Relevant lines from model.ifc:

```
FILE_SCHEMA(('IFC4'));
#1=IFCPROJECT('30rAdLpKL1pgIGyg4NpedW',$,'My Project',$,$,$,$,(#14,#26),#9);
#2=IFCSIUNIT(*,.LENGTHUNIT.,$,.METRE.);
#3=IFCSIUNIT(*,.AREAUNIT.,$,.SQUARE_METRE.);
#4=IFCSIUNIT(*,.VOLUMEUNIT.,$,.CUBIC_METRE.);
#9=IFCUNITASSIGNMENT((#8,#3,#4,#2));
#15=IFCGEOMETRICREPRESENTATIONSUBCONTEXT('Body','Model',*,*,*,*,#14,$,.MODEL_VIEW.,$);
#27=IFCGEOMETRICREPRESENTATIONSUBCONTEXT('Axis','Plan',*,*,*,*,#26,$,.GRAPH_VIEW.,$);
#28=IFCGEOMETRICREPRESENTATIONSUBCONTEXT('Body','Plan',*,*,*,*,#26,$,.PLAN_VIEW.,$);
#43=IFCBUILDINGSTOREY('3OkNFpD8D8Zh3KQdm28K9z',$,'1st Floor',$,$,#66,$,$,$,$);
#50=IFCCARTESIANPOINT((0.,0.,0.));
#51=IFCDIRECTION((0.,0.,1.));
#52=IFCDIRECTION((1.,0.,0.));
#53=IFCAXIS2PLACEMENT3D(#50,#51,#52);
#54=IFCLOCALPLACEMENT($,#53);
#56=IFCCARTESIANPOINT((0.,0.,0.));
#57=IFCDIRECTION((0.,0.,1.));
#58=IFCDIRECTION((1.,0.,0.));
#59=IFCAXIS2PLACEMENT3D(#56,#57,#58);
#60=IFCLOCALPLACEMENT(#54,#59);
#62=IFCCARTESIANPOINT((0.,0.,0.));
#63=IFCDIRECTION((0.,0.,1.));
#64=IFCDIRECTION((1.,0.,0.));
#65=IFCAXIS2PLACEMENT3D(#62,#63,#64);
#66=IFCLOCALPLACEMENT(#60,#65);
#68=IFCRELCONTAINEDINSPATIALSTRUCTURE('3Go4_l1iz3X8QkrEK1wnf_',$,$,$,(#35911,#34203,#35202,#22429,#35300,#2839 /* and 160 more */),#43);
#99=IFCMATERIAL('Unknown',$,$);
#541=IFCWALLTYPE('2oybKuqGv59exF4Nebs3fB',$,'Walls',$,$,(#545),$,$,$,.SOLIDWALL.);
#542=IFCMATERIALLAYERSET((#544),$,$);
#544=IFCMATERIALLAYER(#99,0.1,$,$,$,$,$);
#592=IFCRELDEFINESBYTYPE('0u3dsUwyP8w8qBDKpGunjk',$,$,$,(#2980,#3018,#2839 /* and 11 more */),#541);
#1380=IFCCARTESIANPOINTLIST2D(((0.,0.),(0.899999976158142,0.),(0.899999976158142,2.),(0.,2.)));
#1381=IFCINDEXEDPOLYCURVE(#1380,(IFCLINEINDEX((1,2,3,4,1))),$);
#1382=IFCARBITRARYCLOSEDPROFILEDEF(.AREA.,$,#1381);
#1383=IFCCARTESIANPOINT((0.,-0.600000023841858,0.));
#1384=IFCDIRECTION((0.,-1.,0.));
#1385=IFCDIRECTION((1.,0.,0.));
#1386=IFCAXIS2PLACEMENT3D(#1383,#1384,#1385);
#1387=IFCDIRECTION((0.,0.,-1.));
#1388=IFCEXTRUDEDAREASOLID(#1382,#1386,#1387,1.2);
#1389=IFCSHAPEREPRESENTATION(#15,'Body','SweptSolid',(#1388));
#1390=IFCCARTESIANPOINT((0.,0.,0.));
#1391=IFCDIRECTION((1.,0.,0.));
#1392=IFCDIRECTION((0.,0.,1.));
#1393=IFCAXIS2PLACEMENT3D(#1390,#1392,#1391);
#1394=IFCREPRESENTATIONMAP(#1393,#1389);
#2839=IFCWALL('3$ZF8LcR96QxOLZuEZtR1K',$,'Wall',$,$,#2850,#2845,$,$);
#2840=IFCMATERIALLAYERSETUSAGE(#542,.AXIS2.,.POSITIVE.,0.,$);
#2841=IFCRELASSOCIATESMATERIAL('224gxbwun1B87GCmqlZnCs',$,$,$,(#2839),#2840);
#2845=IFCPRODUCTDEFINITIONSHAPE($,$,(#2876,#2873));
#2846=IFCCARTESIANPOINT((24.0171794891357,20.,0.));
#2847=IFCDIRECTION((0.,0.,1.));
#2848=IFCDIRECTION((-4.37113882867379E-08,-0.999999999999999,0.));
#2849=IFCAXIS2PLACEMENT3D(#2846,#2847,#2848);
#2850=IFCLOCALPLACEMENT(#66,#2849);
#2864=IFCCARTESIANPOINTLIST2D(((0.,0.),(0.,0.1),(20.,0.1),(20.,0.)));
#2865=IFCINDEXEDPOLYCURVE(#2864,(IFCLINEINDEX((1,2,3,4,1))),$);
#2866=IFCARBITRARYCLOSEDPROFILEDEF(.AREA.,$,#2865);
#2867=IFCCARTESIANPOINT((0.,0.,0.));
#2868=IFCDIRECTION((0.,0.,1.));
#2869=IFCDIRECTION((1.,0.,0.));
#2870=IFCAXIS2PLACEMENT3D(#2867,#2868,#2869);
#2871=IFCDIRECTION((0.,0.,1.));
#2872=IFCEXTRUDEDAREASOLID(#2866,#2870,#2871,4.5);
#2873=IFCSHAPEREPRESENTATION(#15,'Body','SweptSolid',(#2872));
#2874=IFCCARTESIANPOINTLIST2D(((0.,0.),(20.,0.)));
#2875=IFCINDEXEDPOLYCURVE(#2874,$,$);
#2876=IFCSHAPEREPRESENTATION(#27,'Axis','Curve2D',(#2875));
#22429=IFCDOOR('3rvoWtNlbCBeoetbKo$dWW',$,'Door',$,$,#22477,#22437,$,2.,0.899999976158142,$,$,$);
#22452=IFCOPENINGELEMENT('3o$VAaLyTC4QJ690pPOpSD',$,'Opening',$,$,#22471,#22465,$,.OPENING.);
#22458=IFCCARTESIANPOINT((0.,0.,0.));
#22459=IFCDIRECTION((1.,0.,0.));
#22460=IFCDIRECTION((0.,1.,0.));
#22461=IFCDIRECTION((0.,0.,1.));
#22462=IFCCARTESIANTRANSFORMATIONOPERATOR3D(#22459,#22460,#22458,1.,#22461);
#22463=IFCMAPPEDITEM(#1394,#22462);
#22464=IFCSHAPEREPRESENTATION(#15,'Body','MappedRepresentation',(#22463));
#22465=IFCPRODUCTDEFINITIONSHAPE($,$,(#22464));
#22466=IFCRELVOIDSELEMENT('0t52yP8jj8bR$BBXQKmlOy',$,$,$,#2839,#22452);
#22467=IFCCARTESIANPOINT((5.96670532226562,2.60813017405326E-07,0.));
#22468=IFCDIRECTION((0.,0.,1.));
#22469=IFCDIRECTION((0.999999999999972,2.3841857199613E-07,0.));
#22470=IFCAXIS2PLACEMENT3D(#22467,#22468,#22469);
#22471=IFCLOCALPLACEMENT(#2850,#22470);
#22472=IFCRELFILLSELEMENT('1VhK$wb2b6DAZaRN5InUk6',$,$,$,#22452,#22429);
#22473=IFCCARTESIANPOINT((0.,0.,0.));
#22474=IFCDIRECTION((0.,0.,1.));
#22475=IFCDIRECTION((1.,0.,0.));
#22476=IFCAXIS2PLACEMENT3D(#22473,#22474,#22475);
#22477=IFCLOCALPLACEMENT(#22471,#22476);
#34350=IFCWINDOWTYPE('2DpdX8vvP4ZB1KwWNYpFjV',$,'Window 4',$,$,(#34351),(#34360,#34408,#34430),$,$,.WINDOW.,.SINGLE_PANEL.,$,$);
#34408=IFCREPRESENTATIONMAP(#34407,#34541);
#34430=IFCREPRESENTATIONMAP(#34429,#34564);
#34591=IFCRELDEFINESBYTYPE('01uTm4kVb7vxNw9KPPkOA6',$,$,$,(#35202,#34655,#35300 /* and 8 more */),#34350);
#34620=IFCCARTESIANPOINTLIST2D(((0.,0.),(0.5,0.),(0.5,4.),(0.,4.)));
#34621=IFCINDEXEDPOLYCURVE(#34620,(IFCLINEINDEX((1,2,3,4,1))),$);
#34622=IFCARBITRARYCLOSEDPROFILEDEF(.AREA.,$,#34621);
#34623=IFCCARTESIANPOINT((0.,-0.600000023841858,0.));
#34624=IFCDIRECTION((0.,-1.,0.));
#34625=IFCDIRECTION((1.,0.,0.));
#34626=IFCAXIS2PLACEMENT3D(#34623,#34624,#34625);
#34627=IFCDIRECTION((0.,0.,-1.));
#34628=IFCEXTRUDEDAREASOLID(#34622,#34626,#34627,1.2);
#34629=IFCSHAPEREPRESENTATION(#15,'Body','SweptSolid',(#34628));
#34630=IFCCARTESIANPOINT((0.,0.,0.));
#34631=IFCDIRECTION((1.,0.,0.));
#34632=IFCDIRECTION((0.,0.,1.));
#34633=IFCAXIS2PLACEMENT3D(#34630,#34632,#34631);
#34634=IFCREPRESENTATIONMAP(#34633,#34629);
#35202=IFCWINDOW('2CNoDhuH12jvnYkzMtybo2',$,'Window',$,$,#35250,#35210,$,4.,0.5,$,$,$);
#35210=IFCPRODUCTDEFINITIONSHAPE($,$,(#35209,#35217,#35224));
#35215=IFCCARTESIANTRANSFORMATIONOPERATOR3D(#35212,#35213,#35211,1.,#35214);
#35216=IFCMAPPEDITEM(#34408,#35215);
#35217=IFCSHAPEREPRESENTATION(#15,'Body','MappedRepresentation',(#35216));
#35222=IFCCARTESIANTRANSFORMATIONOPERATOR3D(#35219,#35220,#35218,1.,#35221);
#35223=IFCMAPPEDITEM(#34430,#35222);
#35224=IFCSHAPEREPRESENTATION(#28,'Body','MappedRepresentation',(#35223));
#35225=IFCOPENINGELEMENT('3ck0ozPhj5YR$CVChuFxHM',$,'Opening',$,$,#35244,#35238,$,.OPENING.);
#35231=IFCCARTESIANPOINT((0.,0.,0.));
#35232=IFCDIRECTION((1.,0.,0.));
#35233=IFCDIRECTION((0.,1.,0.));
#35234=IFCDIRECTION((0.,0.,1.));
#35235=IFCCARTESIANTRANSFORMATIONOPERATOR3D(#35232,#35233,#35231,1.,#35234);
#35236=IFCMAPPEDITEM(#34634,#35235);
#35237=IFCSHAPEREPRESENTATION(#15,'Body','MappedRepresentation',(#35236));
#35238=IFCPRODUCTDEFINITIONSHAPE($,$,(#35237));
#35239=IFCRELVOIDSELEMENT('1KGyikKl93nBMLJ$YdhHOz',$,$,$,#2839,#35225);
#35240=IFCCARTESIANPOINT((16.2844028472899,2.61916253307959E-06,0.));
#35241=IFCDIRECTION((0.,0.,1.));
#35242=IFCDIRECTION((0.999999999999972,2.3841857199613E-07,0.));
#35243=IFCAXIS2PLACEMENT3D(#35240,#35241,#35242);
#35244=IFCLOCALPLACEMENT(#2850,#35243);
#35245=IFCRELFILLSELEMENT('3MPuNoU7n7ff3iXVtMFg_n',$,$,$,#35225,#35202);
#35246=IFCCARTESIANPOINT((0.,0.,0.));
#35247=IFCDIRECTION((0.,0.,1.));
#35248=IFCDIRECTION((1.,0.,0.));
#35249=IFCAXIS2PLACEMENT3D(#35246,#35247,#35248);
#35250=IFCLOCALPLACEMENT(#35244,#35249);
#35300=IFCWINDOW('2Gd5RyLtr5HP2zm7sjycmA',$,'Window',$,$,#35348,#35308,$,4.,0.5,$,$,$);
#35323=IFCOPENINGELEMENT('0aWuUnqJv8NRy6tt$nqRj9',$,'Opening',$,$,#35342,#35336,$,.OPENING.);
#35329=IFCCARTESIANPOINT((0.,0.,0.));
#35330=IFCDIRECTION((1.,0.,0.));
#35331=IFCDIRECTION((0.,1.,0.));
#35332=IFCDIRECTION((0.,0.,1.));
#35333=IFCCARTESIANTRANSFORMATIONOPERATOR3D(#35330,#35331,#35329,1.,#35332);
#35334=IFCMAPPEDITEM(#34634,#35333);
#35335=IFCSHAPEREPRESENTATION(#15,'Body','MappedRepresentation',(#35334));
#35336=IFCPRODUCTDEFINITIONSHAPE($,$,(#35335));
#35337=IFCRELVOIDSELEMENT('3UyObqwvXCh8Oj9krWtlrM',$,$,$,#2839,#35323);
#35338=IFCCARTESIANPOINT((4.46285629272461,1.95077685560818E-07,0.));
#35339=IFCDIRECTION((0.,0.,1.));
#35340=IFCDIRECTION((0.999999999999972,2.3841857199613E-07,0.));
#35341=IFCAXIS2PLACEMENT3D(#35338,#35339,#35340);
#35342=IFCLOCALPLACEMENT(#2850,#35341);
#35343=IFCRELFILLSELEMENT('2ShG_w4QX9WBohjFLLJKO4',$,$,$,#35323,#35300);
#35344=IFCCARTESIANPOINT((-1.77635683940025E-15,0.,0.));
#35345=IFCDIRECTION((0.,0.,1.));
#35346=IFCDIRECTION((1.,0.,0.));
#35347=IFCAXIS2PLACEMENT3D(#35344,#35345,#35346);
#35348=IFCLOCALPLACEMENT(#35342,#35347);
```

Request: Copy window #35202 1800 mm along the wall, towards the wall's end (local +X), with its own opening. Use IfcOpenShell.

```python
import ifcopenshell
import ifcopenshell.api.feature
import ifcopenshell.api.geometry
import ifcopenshell.api.root
import ifcopenshell.geom
import ifcopenshell.util.element
import ifcopenshell.util.placement
import ifcopenshell.util.shape

model = ifcopenshell.open("model.ifc")
settings = ifcopenshell.geom.settings()


def volume(element):
    """Net volume in cubic metres, openings subtracted."""
    shape = ifcopenshell.geom.create_shape(settings, element)
    return ifcopenshell.util.shape.get_volume(shape.geometry)


window = model.by_guid("2CNoDhuH12jvnYkzMtybo2")
opening = window.FillsVoids[0].RelatingOpeningElement
wall = opening.VoidsElements[0].RelatingBuildingElement
before = volume(wall)
shift = ifcopenshell.util.placement.get_local_placement(wall.ObjectPlacement)[:3, 0] * 1.8

# copy_class copies the void relationship, type, container and properties, but no geometry.
new_opening = ifcopenshell.api.root.copy_class(model, product=opening)
new_opening.Representation = ifcopenshell.util.element.copy_deep(
    model, opening.Representation, exclude=["IfcGeometricRepresentationContext", "IfcRepresentationMap"]
)
new_window = ifcopenshell.api.root.copy_class(model, product=window)
new_window.Representation = ifcopenshell.util.element.copy_deep(
    model, window.Representation, exclude=["IfcGeometricRepresentationContext", "IfcRepresentationMap"]
)
ifcopenshell.api.feature.add_filling(model, opening=new_opening, element=new_window)

for old, new in ((opening, new_opening), (window, new_window)):
    matrix = ifcopenshell.util.placement.get_local_placement(old.ObjectPlacement)
    matrix[:3, 3] += shift
    ifcopenshell.api.geometry.edit_object_placement(model, product=new, matrix=matrix, is_si=False)

after = volume(wall)

print(f"wall volume {before:.3f} -> {after:.3f} m3")

model.write("model-out.ifc")
```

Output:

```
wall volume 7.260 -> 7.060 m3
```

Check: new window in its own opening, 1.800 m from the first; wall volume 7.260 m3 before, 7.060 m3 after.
